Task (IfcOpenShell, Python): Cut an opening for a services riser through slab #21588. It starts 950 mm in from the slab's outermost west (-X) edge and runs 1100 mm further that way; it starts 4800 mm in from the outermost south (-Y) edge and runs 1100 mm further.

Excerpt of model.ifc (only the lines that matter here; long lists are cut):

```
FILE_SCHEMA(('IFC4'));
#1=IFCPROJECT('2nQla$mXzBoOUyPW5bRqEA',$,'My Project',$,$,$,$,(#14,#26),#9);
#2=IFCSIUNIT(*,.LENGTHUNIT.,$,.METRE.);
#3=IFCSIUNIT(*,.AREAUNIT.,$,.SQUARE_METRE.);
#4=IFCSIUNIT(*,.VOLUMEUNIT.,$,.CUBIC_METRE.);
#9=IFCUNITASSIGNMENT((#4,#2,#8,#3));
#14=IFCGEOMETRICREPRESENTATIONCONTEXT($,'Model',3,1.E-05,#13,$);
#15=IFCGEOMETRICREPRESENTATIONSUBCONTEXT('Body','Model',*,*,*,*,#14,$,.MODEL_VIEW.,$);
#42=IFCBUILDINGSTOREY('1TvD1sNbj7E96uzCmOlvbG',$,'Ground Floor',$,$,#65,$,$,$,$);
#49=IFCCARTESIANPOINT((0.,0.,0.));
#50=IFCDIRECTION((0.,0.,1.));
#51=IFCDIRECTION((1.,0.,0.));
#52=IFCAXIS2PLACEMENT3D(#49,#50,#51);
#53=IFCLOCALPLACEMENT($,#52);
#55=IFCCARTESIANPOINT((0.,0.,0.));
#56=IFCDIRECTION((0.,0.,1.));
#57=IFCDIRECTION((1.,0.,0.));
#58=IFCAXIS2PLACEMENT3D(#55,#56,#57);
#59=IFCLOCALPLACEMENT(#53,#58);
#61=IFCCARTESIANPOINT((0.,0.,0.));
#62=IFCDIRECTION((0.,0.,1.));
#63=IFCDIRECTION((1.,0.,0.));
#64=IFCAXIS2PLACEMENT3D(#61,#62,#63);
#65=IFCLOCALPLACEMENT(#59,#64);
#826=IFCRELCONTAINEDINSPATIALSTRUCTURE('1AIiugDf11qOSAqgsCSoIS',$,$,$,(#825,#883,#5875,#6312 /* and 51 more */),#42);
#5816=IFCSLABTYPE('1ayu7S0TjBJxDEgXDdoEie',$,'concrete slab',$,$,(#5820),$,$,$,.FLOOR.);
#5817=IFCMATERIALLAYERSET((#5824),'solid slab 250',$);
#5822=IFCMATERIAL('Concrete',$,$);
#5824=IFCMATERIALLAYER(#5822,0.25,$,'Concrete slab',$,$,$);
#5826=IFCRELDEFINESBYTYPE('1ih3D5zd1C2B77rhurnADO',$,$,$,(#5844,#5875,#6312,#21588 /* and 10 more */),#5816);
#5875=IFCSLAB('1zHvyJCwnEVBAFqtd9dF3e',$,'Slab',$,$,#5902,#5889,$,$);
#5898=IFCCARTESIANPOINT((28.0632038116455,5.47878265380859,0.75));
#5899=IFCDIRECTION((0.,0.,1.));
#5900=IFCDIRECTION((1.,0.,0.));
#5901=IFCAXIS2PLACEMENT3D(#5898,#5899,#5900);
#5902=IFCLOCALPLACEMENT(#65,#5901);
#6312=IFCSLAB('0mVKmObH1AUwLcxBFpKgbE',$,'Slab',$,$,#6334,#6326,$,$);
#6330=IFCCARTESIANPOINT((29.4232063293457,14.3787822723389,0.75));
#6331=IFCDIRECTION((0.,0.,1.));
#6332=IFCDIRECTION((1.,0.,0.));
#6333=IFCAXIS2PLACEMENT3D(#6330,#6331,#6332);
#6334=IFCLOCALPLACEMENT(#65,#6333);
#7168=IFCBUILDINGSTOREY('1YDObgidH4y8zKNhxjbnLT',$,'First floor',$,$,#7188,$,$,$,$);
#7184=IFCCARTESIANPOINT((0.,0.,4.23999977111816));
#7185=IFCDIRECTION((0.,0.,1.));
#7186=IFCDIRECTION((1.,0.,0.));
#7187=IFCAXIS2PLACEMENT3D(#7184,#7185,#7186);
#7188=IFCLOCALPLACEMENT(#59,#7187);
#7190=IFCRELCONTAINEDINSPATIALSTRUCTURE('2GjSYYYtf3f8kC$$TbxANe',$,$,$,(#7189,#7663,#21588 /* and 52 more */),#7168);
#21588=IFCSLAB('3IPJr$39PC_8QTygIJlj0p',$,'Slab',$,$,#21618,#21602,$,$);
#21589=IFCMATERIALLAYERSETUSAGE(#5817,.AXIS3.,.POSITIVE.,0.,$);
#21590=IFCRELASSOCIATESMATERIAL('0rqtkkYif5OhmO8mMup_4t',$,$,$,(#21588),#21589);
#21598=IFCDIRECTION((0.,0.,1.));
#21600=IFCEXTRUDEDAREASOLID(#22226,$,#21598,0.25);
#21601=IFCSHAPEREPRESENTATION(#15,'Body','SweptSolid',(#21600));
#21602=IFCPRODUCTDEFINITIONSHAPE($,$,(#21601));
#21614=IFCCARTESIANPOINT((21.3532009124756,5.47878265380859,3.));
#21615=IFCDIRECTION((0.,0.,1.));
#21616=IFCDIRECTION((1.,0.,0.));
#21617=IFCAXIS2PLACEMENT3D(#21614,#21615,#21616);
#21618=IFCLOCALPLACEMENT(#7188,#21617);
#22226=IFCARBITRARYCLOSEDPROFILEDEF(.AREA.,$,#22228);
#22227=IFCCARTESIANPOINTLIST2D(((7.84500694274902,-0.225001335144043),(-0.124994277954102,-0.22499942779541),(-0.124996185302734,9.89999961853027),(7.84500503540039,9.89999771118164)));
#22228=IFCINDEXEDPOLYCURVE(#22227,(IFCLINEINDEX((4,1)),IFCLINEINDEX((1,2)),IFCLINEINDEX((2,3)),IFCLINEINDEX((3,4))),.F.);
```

```python
import numpy as np
import ifcopenshell
import ifcopenshell.api.feature
import ifcopenshell.api.geometry
import ifcopenshell.api.root
import ifcopenshell.geom
import ifcopenshell.util.placement
import ifcopenshell.util.representation
import ifcopenshell.util.shape
import ifcopenshell.util.unit

model = ifcopenshell.open("model.ifc")
unit_scale = ifcopenshell.util.unit.calculate_unit_scale(model)
settings = ifcopenshell.geom.settings()


def volume(element):
    """Net volume in cubic metres, openings subtracted."""
    shape = ifcopenshell.geom.create_shape(settings, element)
    return ifcopenshell.util.shape.get_volume(shape.geometry)


slab = model.by_guid("3IPJr$39PC_8QTygIJlj0p")
before = volume(slab)

# Extent in the slab's own axes, in metres. The edges named are its -X and -Y sides.
slab_shape = ifcopenshell.geom.create_shape(settings, slab)
vertices = ifcopenshell.util.shape.get_vertices(slab_shape.geometry)
x_min, y_min, bottom = vertices.min(axis=0)
top = vertices[:, 2].max()

opening = ifcopenshell.api.root.create_entity(model, ifc_class="IfcOpeningElement", name="Services riser opening", predefined_type="OPENING")
context = ifcopenshell.util.representation.get_context(model, "Model", "Body", "MODEL_VIEW")
width, depth = 1.1, 1.1
outline = [(0.0, 0.0), (width, 0.0), (width, depth), (0.0, depth), (0.0, 0.0)]
# Overshoot both faces by 50 mm so the cut is clean.
shape = ifcopenshell.api.geometry.add_slab_representation(
    model, context=context, depth=top - bottom + 0.1, polyline=outline
)
ifcopenshell.api.geometry.assign_representation(model, product=opening, representation=shape)

matrix = ifcopenshell.util.placement.get_local_placement(slab.ObjectPlacement)
matrix[:, 3] = matrix @ np.append(np.array([x_min + 0.95, y_min + 4.8, bottom - 0.05]) / unit_scale, 1.0)
ifcopenshell.api.geometry.edit_object_placement(model, product=opening, matrix=matrix, is_si=False)
ifcopenshell.api.feature.add_feature(model, feature=opening, element=slab)

after = volume(slab)

print(f"slab volume {before:.3f} -> {after:.3f} m3")

model.write("model_rev.ifc")
```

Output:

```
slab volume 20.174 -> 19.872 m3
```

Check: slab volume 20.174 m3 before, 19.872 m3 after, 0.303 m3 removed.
